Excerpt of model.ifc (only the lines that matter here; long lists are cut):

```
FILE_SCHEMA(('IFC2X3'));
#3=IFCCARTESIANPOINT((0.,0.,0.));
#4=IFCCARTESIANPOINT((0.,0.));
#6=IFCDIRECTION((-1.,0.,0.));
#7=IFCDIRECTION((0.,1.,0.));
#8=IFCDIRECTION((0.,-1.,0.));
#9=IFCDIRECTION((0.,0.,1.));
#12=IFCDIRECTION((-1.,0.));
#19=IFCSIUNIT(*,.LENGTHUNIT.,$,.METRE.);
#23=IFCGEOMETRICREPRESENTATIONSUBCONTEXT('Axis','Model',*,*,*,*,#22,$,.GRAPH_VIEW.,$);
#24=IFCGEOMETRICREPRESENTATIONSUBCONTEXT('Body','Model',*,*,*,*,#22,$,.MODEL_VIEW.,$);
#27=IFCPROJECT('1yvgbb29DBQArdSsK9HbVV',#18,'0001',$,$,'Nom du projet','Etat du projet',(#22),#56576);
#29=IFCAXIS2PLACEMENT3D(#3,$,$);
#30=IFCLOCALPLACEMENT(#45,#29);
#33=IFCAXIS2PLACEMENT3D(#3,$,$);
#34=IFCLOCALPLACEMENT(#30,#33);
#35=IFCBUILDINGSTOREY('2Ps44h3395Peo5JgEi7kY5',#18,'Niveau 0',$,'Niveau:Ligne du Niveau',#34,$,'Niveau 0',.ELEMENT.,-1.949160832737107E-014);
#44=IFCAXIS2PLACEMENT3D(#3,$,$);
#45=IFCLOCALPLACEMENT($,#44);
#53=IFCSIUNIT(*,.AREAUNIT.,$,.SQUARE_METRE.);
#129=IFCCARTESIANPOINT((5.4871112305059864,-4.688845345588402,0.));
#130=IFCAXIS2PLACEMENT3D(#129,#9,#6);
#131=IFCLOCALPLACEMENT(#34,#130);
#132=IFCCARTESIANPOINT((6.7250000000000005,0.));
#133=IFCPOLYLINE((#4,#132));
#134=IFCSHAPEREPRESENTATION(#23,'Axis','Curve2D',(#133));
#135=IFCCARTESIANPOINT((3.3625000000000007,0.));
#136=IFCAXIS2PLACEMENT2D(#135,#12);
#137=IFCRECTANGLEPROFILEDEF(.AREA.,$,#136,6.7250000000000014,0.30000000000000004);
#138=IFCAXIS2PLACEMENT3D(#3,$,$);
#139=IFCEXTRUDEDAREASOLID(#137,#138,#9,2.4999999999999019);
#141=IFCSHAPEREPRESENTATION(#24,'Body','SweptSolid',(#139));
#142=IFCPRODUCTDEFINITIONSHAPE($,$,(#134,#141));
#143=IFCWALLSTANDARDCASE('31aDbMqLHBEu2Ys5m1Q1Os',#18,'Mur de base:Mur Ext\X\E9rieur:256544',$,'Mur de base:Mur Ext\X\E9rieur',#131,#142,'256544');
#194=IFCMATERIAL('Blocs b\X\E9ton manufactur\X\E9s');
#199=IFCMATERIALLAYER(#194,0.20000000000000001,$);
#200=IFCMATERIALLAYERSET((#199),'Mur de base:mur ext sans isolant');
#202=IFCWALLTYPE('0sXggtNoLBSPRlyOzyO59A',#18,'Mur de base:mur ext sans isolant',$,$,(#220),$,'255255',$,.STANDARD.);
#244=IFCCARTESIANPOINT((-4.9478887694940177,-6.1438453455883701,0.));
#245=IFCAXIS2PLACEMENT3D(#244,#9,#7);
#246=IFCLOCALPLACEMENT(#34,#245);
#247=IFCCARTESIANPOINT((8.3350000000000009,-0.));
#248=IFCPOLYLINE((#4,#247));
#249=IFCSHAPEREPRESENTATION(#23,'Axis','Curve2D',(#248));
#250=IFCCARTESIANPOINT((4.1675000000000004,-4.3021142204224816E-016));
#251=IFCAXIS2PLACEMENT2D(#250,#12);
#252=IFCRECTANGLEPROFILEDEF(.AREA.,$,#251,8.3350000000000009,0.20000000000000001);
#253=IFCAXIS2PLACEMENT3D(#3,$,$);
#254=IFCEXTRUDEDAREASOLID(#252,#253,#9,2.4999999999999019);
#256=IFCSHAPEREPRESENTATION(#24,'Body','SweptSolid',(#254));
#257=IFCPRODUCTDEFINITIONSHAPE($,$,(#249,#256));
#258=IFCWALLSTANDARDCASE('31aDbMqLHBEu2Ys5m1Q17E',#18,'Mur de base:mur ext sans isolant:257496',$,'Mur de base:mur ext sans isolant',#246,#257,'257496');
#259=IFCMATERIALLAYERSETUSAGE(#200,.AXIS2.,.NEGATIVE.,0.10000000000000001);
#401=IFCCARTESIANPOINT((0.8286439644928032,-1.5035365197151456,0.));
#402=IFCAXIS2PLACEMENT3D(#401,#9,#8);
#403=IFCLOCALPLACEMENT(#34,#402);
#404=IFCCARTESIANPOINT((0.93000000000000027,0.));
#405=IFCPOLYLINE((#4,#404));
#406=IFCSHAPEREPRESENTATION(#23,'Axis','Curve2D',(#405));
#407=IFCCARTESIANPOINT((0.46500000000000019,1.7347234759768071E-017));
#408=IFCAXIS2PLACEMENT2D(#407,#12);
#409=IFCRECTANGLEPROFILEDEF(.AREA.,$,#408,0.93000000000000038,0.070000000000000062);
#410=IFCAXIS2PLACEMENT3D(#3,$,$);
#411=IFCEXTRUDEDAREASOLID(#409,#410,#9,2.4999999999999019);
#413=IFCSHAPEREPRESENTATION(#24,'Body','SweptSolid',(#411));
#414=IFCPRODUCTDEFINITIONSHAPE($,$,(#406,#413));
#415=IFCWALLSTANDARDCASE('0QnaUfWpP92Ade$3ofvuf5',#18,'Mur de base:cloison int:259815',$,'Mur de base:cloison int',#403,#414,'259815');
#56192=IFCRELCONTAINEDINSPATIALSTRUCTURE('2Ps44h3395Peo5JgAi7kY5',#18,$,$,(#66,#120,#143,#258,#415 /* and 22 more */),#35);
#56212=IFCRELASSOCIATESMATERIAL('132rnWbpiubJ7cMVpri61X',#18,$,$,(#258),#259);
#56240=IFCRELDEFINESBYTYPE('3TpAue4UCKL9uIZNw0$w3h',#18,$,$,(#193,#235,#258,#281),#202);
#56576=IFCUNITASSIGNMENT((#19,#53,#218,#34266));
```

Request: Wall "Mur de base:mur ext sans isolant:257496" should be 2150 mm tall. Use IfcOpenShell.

```python
import ifcopenshell
import ifcopenshell.geom
import ifcopenshell.util.representation
import ifcopenshell.util.shape

model = ifcopenshell.open("model.ifc")
settings = ifcopenshell.geom.settings()


def volume(element):
    """Net volume in cubic metres, openings subtracted."""
    shape = ifcopenshell.geom.create_shape(settings, element)
    return ifcopenshell.util.shape.get_volume(shape.geometry)


wall = model.by_guid("31aDbMqLHBEu2Ys5m1Q17E")
before = volume(wall)

body = ifcopenshell.util.representation.get_representation(wall, "Model", "Body")
solid = body.Items[0]
old_height = solid.Depth
solid.Depth = 2.15
after = volume(wall)

print(f"height {old_height:g} -> {solid.Depth:g}, volume {before:.3f} -> {after:.3f} m3")

model.write("model_edited.ifc")
```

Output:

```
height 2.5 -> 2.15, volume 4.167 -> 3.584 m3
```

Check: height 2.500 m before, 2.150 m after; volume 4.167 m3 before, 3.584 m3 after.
